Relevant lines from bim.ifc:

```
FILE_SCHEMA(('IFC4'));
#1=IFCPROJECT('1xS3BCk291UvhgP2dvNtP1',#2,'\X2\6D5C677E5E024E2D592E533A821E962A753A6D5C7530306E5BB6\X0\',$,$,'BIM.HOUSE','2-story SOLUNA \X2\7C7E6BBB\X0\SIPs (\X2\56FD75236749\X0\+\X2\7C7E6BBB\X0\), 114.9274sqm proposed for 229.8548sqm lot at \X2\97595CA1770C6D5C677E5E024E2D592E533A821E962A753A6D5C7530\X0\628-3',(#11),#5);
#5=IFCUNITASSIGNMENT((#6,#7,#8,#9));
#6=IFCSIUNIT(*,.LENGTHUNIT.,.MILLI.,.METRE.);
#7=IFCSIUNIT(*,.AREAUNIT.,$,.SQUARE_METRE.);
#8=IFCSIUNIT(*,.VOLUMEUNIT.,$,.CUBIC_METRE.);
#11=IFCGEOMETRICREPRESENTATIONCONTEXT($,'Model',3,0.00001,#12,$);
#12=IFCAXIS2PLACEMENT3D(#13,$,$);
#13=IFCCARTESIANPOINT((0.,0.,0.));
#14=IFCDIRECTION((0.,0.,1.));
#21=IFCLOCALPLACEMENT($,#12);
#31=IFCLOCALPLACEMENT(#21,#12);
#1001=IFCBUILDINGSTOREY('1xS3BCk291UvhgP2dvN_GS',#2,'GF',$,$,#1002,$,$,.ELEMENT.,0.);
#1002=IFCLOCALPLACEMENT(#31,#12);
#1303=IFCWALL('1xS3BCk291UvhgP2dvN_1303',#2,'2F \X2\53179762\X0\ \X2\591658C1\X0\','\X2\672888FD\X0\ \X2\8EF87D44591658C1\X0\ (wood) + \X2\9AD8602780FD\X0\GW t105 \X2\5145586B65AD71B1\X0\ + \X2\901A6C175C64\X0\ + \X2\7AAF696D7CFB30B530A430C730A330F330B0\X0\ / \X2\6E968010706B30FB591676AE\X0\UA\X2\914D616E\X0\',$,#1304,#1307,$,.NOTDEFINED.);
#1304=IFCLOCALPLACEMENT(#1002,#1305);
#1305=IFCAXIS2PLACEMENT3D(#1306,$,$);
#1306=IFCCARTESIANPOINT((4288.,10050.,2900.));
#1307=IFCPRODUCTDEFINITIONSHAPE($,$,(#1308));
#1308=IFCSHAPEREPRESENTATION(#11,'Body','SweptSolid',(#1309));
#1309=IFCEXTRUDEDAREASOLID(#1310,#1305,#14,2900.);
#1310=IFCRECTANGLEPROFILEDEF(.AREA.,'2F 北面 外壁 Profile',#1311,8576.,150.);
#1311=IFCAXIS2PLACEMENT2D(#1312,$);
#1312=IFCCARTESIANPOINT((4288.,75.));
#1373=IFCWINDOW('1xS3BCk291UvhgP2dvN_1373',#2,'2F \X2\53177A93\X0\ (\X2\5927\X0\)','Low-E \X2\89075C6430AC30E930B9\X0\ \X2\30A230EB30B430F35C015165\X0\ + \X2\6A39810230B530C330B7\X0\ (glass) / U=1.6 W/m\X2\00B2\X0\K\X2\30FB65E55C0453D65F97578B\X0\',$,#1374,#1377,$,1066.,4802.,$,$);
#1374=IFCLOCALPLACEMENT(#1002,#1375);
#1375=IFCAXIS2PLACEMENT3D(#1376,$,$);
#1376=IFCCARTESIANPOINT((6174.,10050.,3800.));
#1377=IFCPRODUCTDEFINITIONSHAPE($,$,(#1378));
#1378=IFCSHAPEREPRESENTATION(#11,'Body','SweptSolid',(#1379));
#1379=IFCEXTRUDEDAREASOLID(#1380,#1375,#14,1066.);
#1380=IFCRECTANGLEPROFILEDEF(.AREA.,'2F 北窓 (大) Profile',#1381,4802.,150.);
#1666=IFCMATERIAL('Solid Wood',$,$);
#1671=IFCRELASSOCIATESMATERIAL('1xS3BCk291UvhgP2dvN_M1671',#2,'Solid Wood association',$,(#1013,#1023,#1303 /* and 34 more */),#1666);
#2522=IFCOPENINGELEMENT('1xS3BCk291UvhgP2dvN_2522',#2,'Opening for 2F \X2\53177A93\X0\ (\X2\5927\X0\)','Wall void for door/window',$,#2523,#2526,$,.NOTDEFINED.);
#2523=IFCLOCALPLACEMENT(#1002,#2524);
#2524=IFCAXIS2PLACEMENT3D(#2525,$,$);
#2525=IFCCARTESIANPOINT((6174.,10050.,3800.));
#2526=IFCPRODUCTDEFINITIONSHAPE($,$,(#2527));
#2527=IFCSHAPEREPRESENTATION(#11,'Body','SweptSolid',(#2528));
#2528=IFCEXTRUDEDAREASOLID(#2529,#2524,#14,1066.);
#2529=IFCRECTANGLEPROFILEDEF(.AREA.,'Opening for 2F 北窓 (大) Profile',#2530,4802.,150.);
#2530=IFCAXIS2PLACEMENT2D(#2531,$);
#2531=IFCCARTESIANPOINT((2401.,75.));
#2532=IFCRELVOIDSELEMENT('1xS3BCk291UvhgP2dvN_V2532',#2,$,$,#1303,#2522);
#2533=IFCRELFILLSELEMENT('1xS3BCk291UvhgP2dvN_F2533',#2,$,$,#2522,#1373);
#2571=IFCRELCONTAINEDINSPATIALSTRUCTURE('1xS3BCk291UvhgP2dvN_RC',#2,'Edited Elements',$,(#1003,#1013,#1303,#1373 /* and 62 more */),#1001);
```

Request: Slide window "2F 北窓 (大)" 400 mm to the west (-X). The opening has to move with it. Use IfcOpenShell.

```python
import ifcopenshell
import ifcopenshell.api.geometry
import ifcopenshell.util.placement

model = ifcopenshell.open("bim.ifc")

window = model.by_guid("1xS3BCk291UvhgP2dvN_1373")
opening = window.FillsVoids[0].RelatingOpeningElement
wall = opening.VoidsElements[0].RelatingBuildingElement

wall_matrix = ifcopenshell.util.placement.get_local_placement(wall.ObjectPlacement)
shift = wall_matrix[:3, 0] * -400.0
before = ifcopenshell.util.placement.get_local_placement(window.ObjectPlacement)[:3, 3].copy()

# The window is not placed relative to its opening, so move both.
for product in (opening, window):
    matrix = ifcopenshell.util.placement.get_local_placement(product.ObjectPlacement)
    matrix[:3, 3] += shift
    ifcopenshell.api.geometry.edit_object_placement(model, product=product, matrix=matrix, is_si=False)

after = ifcopenshell.util.placement.get_local_placement(window.ObjectPlacement)[:3, 3]
print("window moved by", (after - before).round(3) + 0.0)

model.write("bim_rev.ifc")
```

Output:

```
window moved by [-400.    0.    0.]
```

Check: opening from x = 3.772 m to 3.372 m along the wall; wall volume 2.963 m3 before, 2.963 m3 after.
